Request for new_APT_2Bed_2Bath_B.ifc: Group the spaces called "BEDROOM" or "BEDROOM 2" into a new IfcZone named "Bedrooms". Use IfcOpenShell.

First a look at what the model holds.

```python
import ifcopenshell

model = ifcopenshell.open("new_APT_2Bed_2Bath_B.ifc")
print(model.schema)
seen = {}
for space in model.by_type("IfcSpace"):
    seen[space.LongName] = seen.get(space.LongName, 0) + 1
for name, count in sorted(seen.items(), key=str):
    print(count, "x", name)
print("zones:", [z.Name for z in model.by_type("IfcZone")][:20])
```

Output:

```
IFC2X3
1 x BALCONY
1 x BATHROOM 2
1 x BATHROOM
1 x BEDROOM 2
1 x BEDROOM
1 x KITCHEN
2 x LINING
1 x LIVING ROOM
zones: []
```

```python
import ifcopenshell
import ifcopenshell.api.group
import ifcopenshell.api.root

model = ifcopenshell.open("new_APT_2Bed_2Bath_B.ifc")

names = {"BEDROOM", "BEDROOM 2"}
spaces = [s for s in model.by_type("IfcSpace") if s.LongName in names]

zone = ifcopenshell.api.root.create_entity(model, ifc_class="IfcZone", name="Bedrooms")
ifcopenshell.api.group.assign_group(model, products=spaces, group=zone)
print(len(spaces), "spaces in", zone.Name)

model.write("new_APT_2Bed_2Bath_B_v2.ifc")
```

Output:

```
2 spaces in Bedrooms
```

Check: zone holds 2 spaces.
